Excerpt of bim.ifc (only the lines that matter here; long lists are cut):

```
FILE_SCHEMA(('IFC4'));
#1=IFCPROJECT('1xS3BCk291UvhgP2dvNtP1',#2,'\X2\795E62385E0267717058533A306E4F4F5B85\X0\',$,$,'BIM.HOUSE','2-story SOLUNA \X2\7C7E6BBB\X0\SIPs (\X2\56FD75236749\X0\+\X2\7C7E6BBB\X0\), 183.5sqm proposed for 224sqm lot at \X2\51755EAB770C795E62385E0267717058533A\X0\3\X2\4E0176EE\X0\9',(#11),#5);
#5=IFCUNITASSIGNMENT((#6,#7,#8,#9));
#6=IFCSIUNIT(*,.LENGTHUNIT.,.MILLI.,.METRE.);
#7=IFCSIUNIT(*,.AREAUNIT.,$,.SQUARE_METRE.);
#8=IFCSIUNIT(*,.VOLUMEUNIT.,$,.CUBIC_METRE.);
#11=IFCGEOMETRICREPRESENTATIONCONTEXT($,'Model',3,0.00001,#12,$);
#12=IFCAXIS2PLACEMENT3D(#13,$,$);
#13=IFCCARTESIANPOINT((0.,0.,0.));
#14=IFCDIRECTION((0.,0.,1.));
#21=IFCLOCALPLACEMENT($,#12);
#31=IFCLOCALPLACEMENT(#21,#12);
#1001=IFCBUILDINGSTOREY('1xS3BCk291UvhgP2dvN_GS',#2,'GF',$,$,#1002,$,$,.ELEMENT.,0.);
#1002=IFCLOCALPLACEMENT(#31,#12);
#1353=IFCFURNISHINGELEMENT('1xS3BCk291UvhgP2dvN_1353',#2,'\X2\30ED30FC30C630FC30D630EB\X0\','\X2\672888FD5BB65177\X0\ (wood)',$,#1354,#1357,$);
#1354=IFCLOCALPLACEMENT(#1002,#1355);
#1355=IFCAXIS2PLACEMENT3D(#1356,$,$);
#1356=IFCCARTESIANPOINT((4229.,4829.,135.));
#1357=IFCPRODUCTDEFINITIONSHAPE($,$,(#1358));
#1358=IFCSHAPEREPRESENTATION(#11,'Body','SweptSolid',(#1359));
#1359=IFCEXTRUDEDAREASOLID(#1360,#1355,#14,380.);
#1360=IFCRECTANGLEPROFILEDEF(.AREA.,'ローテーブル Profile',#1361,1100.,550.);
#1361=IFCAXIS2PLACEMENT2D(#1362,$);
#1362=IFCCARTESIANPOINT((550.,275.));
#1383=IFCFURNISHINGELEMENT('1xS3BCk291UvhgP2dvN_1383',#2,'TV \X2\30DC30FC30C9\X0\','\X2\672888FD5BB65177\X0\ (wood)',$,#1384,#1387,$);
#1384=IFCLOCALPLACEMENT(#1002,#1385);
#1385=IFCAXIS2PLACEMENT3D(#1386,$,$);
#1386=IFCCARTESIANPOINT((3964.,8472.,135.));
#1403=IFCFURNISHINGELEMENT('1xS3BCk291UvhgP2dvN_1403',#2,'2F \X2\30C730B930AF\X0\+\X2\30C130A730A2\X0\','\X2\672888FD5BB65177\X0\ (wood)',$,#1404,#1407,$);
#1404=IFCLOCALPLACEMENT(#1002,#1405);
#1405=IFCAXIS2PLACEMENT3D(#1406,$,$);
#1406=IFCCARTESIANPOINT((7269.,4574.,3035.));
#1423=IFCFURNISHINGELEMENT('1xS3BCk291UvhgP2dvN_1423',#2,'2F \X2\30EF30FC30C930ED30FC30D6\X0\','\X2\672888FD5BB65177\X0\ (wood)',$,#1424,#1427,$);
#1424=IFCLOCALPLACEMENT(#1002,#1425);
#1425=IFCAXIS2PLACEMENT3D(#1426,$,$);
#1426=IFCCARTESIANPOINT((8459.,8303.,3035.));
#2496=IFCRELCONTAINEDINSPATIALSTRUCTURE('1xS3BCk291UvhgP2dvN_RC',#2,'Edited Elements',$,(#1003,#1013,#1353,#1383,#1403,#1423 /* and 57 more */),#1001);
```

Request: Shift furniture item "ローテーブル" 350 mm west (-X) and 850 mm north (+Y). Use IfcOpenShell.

```python
import ifcopenshell
import ifcopenshell.api.geometry
import ifcopenshell.util.placement

model = ifcopenshell.open("bim.ifc")

item = model.by_guid("1xS3BCk291UvhgP2dvN_1353")
matrix = ifcopenshell.util.placement.get_local_placement(item.ObjectPlacement)
matrix[0, 3] -= 350.0
matrix[1, 3] += 850.0
ifcopenshell.api.geometry.edit_object_placement(model, product=item, matrix=matrix, is_si=False)

print(ifcopenshell.util.placement.get_local_placement(item.ObjectPlacement).round(3) + 0.0)

model.write("bim_v2.ifc")
```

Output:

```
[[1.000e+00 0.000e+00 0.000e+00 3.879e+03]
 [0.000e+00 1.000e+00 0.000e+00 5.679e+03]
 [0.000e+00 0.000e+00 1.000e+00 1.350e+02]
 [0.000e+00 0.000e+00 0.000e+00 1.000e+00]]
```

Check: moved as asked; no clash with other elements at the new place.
